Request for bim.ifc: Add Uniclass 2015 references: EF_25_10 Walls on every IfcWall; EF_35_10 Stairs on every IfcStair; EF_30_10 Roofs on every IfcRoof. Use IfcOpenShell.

First a look at what the model holds.

```python
import ifcopenshell

model = ifcopenshell.open("bim.ifc")
print(model.schema)
print("classifications:", [c.Name for c in model.by_type("IfcClassification")])
for ifc_class in ("IfcDoor", "IfcRoof", "IfcStair", "IfcWall", "IfcWindow"):
    print(ifc_class, len(model.by_type(ifc_class)))
```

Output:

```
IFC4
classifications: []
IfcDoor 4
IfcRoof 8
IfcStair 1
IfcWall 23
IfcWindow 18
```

```python
import ifcopenshell
import ifcopenshell.api.classification

model = ifcopenshell.open("bim.ifc")

system = ifcopenshell.api.classification.add_classification(model, classification="Uniclass 2015")

codes = {
    "IfcWall": ("EF_25_10", "Walls"),
    "IfcStair": ("EF_35_10", "Stairs"),
    "IfcRoof": ("EF_30_10", "Roofs"),
}
for ifc_class, (code, name) in codes.items():
    products = model.by_type(ifc_class)
    ifcopenshell.api.classification.add_reference(
        model, products=products, classification=system, identification=code, name=name
    )
    print(code, len(products))

model.write("bim_edited.ifc")
```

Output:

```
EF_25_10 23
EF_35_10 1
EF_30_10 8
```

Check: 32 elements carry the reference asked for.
